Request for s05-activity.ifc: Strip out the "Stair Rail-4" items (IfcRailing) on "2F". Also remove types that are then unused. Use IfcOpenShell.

First a look at what the model holds.

```python
import ifcopenshell
import ifcopenshell.util.element

model = ifcopenshell.open("s05-activity.ifc")
print(model.schema)
storey = next(s for s in model.by_type("IfcBuildingStorey") if s.Name == "2F")
railings = [e for e in ifcopenshell.util.element.get_decomposition(storey) if e.is_a("IfcRailing")]
seen = {}
for e in railings:
    element_type = ifcopenshell.util.element.get_type(e)
    name = element_type.Name if element_type not in (None, e) else None
    seen[name] = seen.get(name, 0) + 1
for name, count in sorted(seen.items(), key=str):
    print(count, "x", name)
```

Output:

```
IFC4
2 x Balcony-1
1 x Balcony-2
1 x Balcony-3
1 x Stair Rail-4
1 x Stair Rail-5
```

```python
import ifcopenshell
import ifcopenshell.api.root
import ifcopenshell.util.element

model = ifcopenshell.open("s05-activity.ifc")

storey = next(s for s in model.by_type("IfcBuildingStorey") if s.Name == "2F")
railings = [e for e in ifcopenshell.util.element.get_decomposition(storey) if e.is_a("IfcRailing")]
targets = [e for e in railings if (t := ifcopenshell.util.element.get_type(e)) not in (None, e) and t.Name == "Stair Rail-4"]
types = {ifcopenshell.util.element.get_type(e) for e in targets} - {None, *targets}

for e in targets:
    ifcopenshell.api.root.remove_product(model, product=e)
print(len(targets), "removed")

unused = [t for t in types if not ifcopenshell.util.element.get_types(t)]
for t in unused:
    ifcopenshell.api.root.remove_product(model, product=t)
print(len(unused), "unused types removed")

model.write("s05-activity_rev.ifc")
```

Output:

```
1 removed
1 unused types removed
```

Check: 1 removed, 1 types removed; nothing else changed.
